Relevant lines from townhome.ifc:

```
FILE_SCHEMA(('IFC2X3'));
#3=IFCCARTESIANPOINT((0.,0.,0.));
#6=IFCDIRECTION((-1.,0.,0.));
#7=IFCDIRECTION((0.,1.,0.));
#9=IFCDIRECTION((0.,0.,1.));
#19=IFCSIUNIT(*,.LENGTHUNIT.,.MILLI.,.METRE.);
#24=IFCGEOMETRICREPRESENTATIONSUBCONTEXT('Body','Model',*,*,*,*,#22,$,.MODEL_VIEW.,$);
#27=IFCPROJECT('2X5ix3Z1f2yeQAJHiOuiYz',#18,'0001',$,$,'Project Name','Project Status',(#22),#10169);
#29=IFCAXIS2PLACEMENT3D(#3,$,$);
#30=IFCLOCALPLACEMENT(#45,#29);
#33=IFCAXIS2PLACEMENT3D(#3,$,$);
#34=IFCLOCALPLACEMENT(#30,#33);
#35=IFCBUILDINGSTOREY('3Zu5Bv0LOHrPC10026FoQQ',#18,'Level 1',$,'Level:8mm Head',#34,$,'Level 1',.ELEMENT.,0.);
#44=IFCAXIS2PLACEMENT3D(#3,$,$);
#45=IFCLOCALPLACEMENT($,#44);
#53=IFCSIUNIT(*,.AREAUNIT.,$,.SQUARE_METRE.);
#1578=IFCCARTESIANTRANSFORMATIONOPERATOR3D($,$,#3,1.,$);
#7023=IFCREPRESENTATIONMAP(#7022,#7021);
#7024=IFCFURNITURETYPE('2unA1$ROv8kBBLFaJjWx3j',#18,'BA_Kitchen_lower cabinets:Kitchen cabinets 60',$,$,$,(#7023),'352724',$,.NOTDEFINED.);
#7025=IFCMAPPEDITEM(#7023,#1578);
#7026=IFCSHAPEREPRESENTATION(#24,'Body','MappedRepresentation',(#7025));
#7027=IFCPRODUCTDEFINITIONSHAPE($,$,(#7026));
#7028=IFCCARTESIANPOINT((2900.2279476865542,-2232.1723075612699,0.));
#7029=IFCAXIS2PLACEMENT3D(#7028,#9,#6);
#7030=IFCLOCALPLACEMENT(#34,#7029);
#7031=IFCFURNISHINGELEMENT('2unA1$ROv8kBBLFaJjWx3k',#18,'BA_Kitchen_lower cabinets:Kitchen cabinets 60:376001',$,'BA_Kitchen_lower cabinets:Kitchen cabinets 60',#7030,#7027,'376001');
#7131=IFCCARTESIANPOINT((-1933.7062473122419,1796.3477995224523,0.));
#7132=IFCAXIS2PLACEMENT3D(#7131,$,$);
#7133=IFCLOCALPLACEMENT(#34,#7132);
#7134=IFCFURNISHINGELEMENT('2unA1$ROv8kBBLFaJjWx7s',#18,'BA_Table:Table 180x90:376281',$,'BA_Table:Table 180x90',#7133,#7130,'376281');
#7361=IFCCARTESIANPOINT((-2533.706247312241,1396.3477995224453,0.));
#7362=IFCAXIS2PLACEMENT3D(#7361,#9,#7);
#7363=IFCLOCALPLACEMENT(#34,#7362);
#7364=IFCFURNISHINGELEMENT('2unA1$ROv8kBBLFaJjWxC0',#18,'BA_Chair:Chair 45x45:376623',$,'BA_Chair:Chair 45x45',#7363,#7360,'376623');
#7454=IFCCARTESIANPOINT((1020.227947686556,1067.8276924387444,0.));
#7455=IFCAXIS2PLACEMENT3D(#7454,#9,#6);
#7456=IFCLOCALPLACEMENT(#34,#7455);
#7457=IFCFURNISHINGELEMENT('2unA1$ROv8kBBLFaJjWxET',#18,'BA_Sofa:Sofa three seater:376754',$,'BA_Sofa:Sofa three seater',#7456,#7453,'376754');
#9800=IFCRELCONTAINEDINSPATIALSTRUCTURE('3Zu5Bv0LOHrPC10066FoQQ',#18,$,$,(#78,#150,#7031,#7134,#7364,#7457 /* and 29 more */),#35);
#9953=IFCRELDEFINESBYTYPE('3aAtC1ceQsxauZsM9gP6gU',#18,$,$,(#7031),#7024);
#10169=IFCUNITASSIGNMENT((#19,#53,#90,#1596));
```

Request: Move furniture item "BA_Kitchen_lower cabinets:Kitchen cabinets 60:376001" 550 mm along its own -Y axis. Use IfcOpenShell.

```python
import ifcopenshell
import ifcopenshell.api.geometry
import ifcopenshell.util.placement
import ifcopenshell.util.unit

model = ifcopenshell.open("townhome.ifc")
unit_scale = ifcopenshell.util.unit.calculate_unit_scale(model)

item = model.by_id(7031)
matrix = ifcopenshell.util.placement.get_local_placement(item.ObjectPlacement)
matrix[:3, 3] -= matrix[:3, 1] * 0.55 / unit_scale
ifcopenshell.api.geometry.edit_object_placement(model, product=item, matrix=matrix, is_si=False)

print(ifcopenshell.util.placement.get_local_placement(item.ObjectPlacement).round(3) + 0.0)

model.write("townhome_v2.ifc")
```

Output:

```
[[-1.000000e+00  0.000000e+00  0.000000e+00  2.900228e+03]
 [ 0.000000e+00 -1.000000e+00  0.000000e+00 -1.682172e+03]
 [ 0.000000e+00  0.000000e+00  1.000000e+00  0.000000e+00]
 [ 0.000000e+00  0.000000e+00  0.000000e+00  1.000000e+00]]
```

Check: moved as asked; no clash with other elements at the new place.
